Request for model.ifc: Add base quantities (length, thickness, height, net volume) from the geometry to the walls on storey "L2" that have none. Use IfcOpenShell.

First a look at what the model holds.

```python
import ifcopenshell
import ifcopenshell.util.element
import ifcopenshell.util.unit

model = ifcopenshell.open("model.ifc")
print(model.schema)
for unit_type in ("LENGTHUNIT", "AREAUNIT", "VOLUMEUNIT"):
    print(unit_type, ifcopenshell.util.unit.calculate_unit_scale(model, unit_type))
storey = next(s for s in model.by_type("IfcBuildingStorey") if s.Name == "L2")
walls = [e for e in ifcopenshell.util.element.get_decomposition(storey) if e.is_a("IfcWall")]
for e in sorted(walls, key=lambda e: e.id()):
    print(e.id(), e.is_a(), e.Name, list(ifcopenshell.util.element.get_psets(e, qtos_only=True)), sep=" | ")
```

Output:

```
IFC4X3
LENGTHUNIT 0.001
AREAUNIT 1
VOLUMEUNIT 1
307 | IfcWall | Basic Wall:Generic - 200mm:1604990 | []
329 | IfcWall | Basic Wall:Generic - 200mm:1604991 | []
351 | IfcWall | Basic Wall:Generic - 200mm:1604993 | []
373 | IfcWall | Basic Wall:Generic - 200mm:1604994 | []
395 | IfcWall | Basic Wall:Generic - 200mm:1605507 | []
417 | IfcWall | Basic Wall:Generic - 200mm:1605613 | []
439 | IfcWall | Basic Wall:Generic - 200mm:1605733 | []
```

```python
import ifcopenshell
import ifcopenshell.api.pset
import ifcopenshell.geom
import ifcopenshell.util.element
import ifcopenshell.util.shape
import ifcopenshell.util.unit

model = ifcopenshell.open("model.ifc")
unit_scale = ifcopenshell.util.unit.calculate_unit_scale(model)
volume_scale = ifcopenshell.util.unit.calculate_unit_scale(model, "VOLUMEUNIT")
settings = ifcopenshell.geom.settings()

storey = next(s for s in model.by_type("IfcBuildingStorey") if s.Name == "L2")
walls = [e for e in ifcopenshell.util.element.get_decomposition(storey) if e.is_a("IfcWall")]

for e in sorted(walls, key=lambda e: e.id()):
    if ifcopenshell.util.element.get_psets(e, qtos_only=True, should_inherit=False):
        continue
    # Geometry comes back in metres, in the element's own axes.
    shape = ifcopenshell.geom.create_shape(settings, e)
    values = {
        "Length": ifcopenshell.util.shape.get_x(shape.geometry) / unit_scale,
        "Width": ifcopenshell.util.shape.get_y(shape.geometry) / unit_scale,
        "Height": ifcopenshell.util.shape.get_z(shape.geometry) / unit_scale,
        "NetVolume": ifcopenshell.util.shape.get_volume(shape.geometry) / volume_scale,
    }
    qto = ifcopenshell.api.pset.add_qto(model, product=e, name="Qto_WallBaseQuantities")
    ifcopenshell.api.pset.edit_qto(model, qto=qto, properties=values)
    print(e.id(), {k: round(v, 3) for k, v in values.items()})

model.write("model_rev.ifc")
```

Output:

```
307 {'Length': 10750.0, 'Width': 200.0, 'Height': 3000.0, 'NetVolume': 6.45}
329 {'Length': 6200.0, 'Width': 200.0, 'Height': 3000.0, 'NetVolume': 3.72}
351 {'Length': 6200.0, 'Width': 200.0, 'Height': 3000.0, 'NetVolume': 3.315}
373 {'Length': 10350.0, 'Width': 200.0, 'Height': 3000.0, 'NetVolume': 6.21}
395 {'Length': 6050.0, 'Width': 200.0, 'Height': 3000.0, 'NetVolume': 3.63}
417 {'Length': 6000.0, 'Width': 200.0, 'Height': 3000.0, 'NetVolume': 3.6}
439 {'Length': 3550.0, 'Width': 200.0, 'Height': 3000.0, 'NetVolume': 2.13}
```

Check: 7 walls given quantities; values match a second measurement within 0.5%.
